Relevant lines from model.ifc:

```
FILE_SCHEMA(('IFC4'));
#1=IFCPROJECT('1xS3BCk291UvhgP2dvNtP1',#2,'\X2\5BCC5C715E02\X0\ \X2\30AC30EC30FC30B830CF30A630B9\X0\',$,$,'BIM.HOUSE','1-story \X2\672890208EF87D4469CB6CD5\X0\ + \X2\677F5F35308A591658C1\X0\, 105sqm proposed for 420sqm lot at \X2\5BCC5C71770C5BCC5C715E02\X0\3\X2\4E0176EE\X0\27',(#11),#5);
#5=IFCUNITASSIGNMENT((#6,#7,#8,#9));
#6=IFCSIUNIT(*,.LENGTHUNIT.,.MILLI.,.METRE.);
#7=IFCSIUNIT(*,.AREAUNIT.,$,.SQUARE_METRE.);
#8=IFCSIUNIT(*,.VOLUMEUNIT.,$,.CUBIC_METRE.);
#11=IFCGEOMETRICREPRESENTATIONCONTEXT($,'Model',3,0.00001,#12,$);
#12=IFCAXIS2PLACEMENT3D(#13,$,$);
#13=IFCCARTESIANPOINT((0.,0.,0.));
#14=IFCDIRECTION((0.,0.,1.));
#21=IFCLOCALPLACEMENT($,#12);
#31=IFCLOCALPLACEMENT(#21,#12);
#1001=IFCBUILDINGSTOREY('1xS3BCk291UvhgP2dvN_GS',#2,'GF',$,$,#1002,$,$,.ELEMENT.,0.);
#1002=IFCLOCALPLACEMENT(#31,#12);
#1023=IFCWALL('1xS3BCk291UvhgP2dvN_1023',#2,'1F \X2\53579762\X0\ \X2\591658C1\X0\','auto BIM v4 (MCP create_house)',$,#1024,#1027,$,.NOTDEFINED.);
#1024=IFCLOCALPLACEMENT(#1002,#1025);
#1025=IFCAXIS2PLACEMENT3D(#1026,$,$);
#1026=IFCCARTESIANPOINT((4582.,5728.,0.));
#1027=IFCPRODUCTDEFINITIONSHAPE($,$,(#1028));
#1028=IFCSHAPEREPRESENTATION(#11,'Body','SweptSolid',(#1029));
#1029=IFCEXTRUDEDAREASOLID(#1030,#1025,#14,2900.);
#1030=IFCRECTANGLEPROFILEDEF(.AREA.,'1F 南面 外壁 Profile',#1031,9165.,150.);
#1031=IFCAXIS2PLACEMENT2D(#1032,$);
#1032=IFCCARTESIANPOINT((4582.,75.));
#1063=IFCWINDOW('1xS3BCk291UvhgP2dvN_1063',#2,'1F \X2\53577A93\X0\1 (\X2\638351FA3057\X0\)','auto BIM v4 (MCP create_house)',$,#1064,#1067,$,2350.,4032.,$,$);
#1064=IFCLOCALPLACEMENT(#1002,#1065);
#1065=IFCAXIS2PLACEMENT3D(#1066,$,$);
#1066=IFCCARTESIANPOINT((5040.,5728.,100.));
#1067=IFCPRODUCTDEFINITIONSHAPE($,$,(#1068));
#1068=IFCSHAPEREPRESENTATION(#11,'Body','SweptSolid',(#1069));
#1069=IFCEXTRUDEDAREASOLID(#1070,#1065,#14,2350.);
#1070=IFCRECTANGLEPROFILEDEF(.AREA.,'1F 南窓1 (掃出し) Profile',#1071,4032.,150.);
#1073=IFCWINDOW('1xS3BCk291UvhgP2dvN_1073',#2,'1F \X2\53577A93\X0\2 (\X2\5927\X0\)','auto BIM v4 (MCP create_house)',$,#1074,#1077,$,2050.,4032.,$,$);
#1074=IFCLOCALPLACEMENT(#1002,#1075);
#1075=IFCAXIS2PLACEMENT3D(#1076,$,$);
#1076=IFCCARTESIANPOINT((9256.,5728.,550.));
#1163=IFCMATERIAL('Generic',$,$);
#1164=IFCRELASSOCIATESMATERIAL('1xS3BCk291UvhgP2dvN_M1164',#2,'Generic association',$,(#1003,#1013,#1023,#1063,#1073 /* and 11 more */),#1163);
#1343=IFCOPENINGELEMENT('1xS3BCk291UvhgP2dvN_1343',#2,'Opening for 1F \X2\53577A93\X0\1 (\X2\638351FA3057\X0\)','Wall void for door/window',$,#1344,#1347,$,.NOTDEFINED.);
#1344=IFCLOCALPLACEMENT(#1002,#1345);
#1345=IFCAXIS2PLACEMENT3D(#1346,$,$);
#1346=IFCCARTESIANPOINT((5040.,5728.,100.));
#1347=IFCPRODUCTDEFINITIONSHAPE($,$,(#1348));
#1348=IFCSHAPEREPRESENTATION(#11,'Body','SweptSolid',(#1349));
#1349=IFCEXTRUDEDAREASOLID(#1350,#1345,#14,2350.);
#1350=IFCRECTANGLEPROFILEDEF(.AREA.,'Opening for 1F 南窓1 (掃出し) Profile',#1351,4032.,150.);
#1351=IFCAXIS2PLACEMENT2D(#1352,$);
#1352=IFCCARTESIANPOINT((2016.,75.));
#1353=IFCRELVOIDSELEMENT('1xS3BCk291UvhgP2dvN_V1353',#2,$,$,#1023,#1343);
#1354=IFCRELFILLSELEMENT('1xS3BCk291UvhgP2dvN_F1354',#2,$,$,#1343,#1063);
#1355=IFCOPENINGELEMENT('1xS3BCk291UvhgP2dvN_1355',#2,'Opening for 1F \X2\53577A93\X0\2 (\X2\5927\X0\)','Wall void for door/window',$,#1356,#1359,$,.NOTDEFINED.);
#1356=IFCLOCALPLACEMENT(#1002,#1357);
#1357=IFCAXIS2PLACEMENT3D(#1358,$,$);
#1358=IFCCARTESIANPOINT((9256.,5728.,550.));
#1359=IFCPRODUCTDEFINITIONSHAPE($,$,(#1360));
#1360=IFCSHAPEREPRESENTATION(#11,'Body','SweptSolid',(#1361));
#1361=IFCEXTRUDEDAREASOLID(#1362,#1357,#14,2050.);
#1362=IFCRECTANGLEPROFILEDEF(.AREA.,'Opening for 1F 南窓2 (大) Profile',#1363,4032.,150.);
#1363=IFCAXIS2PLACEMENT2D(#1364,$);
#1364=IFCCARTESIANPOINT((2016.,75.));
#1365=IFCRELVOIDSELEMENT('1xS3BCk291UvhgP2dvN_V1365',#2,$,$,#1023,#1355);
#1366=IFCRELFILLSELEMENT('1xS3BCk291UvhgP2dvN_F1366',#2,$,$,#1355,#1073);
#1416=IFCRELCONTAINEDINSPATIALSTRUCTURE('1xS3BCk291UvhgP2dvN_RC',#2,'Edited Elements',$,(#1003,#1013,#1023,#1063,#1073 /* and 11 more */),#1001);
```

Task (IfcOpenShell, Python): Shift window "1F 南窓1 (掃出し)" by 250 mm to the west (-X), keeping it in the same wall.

```python
import ifcopenshell
import ifcopenshell.api.geometry
import ifcopenshell.util.placement

model = ifcopenshell.open("model.ifc")

window = model.by_guid("1xS3BCk291UvhgP2dvN_1063")
opening = window.FillsVoids[0].RelatingOpeningElement
wall = opening.VoidsElements[0].RelatingBuildingElement

wall_matrix = ifcopenshell.util.placement.get_local_placement(wall.ObjectPlacement)
shift = wall_matrix[:3, 0] * -250.0
before = ifcopenshell.util.placement.get_local_placement(window.ObjectPlacement)[:3, 3].copy()

# The window is not placed relative to its opening, so move both.
for product in (opening, window):
    matrix = ifcopenshell.util.placement.get_local_placement(product.ObjectPlacement)
    matrix[:3, 3] += shift
    ifcopenshell.api.geometry.edit_object_placement(model, product=product, matrix=matrix, is_si=False)

after = ifcopenshell.util.placement.get_local_placement(window.ObjectPlacement)[:3, 3]
print("window moved by", (after - before).round(3) + 0.0)

model.write("model-out.ifc")
```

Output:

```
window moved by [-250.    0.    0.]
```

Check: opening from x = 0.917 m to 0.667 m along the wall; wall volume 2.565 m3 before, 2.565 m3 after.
